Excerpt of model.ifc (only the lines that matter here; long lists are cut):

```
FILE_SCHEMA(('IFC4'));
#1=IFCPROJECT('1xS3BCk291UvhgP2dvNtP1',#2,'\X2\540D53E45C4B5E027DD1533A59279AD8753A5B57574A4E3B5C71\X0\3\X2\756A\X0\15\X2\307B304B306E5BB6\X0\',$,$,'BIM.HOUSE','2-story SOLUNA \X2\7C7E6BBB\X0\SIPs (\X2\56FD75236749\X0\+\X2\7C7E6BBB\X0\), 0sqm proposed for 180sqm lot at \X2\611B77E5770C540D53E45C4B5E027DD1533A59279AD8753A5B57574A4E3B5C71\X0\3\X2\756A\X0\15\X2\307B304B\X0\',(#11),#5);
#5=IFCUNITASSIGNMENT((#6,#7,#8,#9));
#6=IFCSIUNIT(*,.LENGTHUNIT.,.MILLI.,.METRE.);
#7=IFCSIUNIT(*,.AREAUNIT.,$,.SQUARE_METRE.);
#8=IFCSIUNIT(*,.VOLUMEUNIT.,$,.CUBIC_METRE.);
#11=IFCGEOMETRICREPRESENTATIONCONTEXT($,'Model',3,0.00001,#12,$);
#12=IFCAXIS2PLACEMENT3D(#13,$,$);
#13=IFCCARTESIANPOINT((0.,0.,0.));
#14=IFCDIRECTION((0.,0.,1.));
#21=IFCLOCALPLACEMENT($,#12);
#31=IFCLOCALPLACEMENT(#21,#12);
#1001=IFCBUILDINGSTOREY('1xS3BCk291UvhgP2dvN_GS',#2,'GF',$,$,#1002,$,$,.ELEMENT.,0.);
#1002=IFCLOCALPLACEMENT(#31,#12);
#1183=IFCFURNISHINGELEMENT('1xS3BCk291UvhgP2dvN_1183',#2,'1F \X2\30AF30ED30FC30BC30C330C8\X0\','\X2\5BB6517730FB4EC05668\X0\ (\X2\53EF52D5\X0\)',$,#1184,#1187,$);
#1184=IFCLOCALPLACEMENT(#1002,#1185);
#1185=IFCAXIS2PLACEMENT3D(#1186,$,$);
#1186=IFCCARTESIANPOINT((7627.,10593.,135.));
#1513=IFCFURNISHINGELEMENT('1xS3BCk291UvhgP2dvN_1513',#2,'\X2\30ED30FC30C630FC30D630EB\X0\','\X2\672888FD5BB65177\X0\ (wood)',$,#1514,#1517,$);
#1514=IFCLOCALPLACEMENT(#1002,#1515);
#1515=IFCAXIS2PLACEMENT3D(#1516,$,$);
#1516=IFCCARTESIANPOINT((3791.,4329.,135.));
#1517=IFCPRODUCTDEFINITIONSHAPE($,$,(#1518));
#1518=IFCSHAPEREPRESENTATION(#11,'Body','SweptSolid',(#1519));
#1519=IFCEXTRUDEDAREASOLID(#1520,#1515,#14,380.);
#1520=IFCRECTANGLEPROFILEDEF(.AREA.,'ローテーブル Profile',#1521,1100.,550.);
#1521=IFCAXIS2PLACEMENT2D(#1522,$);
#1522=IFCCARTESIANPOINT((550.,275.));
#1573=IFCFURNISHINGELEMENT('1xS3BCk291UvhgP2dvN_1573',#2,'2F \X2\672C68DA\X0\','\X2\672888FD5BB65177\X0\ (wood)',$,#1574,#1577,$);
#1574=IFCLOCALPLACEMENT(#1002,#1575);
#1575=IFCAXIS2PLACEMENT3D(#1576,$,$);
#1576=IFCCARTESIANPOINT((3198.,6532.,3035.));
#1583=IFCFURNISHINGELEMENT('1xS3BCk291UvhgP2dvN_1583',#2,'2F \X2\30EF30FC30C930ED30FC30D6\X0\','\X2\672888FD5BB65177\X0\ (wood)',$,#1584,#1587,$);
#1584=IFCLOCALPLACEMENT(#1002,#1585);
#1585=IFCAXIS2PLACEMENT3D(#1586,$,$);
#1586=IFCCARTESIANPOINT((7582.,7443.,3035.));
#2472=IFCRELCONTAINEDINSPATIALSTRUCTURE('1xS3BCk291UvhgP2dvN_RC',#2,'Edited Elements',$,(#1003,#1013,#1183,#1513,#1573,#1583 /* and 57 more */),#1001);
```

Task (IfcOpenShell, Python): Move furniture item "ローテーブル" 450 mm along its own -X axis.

```python
import ifcopenshell
import ifcopenshell.api.geometry
import ifcopenshell.util.placement
import ifcopenshell.util.unit

model = ifcopenshell.open("model.ifc")
unit_scale = ifcopenshell.util.unit.calculate_unit_scale(model)

item = model.by_id(1513)
matrix = ifcopenshell.util.placement.get_local_placement(item.ObjectPlacement)
matrix[:3, 3] -= matrix[:3, 0] * 0.45 / unit_scale
ifcopenshell.api.geometry.edit_object_placement(model, product=item, matrix=matrix, is_si=False)

print(ifcopenshell.util.placement.get_local_placement(item.ObjectPlacement).round(3) + 0.0)

model.write("model_v2.ifc")
```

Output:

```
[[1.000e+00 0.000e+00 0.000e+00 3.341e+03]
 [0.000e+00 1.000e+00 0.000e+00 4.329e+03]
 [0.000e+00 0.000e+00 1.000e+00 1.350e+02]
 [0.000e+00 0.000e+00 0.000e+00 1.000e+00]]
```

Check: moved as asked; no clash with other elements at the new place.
